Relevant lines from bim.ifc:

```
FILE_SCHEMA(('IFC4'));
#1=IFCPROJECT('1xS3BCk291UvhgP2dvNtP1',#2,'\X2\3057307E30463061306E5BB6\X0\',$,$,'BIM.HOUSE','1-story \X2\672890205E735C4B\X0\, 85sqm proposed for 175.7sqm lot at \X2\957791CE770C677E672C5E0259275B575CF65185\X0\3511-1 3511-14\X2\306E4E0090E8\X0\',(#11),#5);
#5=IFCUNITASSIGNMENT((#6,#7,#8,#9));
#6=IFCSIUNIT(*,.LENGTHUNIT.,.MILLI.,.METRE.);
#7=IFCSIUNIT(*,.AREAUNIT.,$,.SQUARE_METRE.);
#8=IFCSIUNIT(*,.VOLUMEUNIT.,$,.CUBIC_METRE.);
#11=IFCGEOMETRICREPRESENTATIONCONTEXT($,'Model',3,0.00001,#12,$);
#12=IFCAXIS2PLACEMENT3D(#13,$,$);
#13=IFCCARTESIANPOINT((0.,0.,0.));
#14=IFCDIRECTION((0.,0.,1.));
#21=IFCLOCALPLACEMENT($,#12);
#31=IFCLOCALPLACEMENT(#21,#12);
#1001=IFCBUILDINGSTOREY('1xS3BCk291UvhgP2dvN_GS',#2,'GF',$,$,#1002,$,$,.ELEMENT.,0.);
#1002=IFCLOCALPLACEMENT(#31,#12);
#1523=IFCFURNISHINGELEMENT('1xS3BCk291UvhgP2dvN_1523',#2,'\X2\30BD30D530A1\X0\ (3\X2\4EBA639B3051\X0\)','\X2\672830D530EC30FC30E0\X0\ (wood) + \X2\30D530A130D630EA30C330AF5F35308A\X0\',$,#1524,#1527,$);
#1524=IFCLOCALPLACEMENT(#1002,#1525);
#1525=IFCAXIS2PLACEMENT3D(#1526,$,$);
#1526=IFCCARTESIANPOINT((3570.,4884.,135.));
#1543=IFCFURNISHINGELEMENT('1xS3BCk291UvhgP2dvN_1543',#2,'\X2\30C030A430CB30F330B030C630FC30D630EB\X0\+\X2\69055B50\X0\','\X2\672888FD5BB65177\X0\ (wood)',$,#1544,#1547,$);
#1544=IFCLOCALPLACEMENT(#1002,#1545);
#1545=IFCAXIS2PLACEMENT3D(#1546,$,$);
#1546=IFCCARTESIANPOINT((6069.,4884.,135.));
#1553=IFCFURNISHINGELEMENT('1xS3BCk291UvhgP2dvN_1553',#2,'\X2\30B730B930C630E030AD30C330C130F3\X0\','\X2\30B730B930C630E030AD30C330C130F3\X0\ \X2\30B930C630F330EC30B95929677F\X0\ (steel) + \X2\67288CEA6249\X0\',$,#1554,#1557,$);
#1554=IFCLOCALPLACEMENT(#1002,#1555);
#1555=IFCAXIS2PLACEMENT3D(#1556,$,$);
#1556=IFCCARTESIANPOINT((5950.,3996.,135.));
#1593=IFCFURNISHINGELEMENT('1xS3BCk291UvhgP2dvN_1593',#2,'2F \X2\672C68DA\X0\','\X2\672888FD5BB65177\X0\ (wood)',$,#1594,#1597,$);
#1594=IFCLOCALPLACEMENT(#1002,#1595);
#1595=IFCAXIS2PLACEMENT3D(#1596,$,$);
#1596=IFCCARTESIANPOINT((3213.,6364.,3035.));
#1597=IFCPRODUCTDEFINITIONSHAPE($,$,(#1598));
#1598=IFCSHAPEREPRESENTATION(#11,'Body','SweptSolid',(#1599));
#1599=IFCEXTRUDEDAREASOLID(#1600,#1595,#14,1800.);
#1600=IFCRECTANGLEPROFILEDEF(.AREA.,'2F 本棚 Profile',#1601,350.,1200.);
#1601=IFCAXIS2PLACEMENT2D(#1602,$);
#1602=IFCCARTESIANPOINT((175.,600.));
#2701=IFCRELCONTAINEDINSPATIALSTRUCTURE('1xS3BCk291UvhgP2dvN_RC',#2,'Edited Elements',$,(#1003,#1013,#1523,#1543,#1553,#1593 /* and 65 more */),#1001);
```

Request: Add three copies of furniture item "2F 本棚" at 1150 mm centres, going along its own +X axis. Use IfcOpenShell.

```python
import ifcopenshell
import ifcopenshell.api.geometry
import ifcopenshell.api.root
import ifcopenshell.util.element
import ifcopenshell.util.placement

model = ifcopenshell.open("bim.ifc")


def reuse_history(source, copy):
    """copy_class also copies each property set's owner history, people and application; keep the originals."""
    for rel in copy.IsDefinedBy:
        if rel.is_a("IfcRelDefinesByProperties") and (history := rel.RelatingPropertyDefinition.OwnerHistory):
            rel.RelatingPropertyDefinition.OwnerHistory = source.OwnerHistory
            ifcopenshell.util.element.remove_deep2(model, history)


source = model.by_guid("1xS3BCk291UvhgP2dvN_1593")
base = ifcopenshell.util.placement.get_local_placement(source.ObjectPlacement)
step = base[:3, 0] * 1150.0

for i in range(1, 4):
    copy = ifcopenshell.api.root.copy_class(model, product=source)
    copy.Representation = ifcopenshell.util.element.copy_deep(
        model, source.Representation, exclude=["IfcGeometricRepresentationContext", "IfcRepresentationMap"]
    )
    reuse_history(source, copy)
    matrix = base.copy()
    matrix[:3, 3] += i * step
    print("added at", matrix[:3, 3].round(3) + 0.0)
    ifcopenshell.api.geometry.edit_object_placement(model, product=copy, matrix=matrix, is_si=False)

model.write("bim_v2.ifc")
```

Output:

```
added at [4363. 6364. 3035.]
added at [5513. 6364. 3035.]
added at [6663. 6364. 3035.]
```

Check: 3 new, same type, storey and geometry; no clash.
